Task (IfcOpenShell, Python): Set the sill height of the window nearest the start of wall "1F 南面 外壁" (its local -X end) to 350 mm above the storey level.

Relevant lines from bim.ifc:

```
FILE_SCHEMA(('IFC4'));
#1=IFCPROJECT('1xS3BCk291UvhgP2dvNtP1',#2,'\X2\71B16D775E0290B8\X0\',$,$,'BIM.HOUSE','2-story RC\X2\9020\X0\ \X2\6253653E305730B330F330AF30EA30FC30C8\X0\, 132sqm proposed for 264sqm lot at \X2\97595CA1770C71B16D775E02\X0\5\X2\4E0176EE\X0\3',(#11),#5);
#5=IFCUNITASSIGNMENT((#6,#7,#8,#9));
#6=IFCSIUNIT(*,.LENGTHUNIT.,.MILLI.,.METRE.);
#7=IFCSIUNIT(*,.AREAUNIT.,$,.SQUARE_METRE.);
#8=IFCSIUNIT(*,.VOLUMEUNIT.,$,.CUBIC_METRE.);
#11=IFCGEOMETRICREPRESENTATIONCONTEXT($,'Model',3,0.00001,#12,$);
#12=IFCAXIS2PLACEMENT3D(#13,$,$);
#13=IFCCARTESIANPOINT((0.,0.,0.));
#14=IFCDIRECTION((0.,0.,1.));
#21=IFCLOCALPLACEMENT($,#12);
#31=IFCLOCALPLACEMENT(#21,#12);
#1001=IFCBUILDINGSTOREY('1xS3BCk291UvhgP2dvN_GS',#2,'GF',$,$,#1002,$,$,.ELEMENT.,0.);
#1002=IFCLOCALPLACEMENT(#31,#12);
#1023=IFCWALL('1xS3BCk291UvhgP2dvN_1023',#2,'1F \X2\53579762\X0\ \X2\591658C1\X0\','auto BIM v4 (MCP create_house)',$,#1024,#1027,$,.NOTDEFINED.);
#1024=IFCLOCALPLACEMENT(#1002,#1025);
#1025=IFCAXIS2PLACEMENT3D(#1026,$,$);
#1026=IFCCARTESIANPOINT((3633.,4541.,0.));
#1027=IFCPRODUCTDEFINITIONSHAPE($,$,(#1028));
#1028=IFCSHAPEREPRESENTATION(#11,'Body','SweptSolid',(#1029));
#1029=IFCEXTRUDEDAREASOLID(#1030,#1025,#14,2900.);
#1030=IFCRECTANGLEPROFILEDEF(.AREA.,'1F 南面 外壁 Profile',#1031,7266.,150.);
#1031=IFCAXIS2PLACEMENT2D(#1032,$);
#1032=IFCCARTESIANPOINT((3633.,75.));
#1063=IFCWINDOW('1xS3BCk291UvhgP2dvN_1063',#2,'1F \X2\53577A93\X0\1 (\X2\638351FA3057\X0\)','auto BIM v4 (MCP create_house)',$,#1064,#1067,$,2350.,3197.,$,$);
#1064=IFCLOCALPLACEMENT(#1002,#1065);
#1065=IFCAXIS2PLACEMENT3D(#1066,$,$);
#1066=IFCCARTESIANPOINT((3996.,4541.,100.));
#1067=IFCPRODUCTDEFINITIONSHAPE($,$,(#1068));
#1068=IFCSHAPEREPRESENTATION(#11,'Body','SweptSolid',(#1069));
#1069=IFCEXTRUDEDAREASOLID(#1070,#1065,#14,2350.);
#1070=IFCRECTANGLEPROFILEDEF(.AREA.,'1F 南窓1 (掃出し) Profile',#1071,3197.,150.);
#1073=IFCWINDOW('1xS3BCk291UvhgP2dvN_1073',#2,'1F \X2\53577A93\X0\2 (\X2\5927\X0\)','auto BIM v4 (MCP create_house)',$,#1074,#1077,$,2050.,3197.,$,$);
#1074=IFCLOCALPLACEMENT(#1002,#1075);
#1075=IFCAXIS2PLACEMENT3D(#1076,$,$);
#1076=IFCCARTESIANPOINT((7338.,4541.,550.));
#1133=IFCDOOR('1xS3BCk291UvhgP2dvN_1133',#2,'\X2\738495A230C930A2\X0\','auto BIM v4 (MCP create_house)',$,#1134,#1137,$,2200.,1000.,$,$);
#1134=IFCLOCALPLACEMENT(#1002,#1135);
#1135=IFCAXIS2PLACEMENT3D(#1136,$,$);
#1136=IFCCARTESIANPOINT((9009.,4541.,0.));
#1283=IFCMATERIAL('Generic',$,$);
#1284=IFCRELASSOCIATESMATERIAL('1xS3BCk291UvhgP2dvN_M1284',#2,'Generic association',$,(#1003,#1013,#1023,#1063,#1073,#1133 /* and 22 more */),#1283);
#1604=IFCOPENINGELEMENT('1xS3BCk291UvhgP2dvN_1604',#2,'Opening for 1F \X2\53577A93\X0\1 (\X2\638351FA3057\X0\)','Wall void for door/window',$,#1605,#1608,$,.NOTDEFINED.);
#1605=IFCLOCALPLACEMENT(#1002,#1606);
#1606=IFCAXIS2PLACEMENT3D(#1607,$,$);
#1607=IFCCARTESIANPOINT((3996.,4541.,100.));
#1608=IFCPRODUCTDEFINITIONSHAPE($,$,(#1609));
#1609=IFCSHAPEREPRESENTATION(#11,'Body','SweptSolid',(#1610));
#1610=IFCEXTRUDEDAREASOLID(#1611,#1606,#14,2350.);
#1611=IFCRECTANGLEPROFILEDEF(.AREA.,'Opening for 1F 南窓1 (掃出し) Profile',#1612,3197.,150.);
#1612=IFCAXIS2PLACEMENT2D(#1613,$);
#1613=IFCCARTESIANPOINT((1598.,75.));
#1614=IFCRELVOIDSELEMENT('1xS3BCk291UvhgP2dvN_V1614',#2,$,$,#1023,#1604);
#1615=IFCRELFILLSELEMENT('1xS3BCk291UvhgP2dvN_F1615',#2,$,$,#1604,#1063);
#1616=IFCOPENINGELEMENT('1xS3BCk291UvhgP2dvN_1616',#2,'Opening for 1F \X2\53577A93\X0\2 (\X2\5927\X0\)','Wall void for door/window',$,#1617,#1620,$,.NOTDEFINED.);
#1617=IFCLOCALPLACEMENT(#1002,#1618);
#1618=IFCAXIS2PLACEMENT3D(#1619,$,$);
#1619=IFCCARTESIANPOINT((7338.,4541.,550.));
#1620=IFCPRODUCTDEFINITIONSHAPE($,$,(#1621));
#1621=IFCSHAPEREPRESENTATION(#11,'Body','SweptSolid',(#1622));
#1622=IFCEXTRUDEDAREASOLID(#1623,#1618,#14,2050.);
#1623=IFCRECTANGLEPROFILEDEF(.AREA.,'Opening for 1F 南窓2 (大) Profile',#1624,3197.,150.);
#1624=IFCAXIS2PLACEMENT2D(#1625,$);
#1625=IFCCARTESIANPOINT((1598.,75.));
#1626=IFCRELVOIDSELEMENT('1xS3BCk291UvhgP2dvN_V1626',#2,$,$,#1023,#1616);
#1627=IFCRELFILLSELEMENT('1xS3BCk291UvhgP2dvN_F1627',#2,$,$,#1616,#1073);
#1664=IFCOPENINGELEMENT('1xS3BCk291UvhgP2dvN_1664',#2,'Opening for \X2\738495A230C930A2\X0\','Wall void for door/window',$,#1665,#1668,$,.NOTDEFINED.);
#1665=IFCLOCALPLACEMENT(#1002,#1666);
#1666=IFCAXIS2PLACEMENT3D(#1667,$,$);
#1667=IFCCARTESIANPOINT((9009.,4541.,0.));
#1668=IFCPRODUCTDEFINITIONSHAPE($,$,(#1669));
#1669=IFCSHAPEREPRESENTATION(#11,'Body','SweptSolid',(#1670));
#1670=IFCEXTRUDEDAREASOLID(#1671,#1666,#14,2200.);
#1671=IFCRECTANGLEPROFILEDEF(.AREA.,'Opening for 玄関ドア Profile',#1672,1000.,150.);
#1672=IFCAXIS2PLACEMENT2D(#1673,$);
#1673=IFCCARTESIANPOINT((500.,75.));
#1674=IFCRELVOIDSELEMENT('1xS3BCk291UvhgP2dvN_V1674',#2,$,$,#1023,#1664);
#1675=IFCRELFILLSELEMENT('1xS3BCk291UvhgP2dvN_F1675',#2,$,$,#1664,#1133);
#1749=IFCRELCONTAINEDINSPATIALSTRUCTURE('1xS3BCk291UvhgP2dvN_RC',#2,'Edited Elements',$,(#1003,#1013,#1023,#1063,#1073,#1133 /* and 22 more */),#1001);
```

```python
import numpy as np
import ifcopenshell
import ifcopenshell.api.geometry
import ifcopenshell.geom
import ifcopenshell.util.element
import ifcopenshell.util.placement
import ifcopenshell.util.shape
import ifcopenshell.util.unit

model = ifcopenshell.open("bim.ifc")
unit_scale = ifcopenshell.util.unit.calculate_unit_scale(model)

window = model.by_guid("1xS3BCk291UvhgP2dvN_1063")
opening = window.FillsVoids[0].RelatingOpeningElement
storey = ifcopenshell.util.element.get_container(window, ifc_class="IfcBuildingStorey")
level = ifcopenshell.util.placement.get_local_placement(storey.ObjectPlacement)[2, 3]

# The opening's origin need not be at the sill, so measure its lowest point.
shape = ifcopenshell.geom.create_shape(ifcopenshell.geom.settings(), opening)
bottom = ifcopenshell.util.shape.get_shape_bottom_elevation(shape, shape.geometry) / unit_scale
dz = level + 0.35 / unit_scale - bottom

shift = np.array([0.0, 0.0, dz])
# The window is not placed relative to its opening, so move both.
for product in (opening, window):
    matrix = ifcopenshell.util.placement.get_local_placement(product.ObjectPlacement)
    matrix[:3, 3] += shift
    ifcopenshell.api.geometry.edit_object_placement(model, product=product, matrix=matrix, is_si=False)

print(f"moved by {dz * unit_scale:+.3f} m")

model.write("bim_edited.ifc")
```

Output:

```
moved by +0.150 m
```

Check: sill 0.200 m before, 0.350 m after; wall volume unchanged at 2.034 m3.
